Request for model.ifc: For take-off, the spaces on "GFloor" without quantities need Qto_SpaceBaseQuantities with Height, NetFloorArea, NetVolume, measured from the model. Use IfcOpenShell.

First a look at what the model holds.

```python
import ifcopenshell
import ifcopenshell.util.element
import ifcopenshell.util.unit

model = ifcopenshell.open("model.ifc")
print(model.schema)
for unit_type in ("LENGTHUNIT", "AREAUNIT", "VOLUMEUNIT"):
    print(unit_type, ifcopenshell.util.unit.calculate_unit_scale(model, unit_type))
storey = next(s for s in model.by_type("IfcBuildingStorey") if s.Name == "GFloor")
spaces = [e for e in ifcopenshell.util.element.get_decomposition(storey) if e.is_a("IfcSpace")]
for e in sorted(spaces, key=lambda e: e.id()):
    print(e.id(), e.is_a(), e.Name, list(ifcopenshell.util.element.get_psets(e, qtos_only=True)), sep=" | ")
```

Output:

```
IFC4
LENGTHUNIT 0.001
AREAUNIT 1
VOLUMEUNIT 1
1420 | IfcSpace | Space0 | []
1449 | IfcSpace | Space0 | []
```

```python
import ifcopenshell
import ifcopenshell.api.pset
import ifcopenshell.geom
import ifcopenshell.util.element
import ifcopenshell.util.shape
import ifcopenshell.util.unit

model = ifcopenshell.open("model.ifc")
unit_scale = ifcopenshell.util.unit.calculate_unit_scale(model)
area_scale = ifcopenshell.util.unit.calculate_unit_scale(model, "AREAUNIT")
volume_scale = ifcopenshell.util.unit.calculate_unit_scale(model, "VOLUMEUNIT")
settings = ifcopenshell.geom.settings()

storey = next(s for s in model.by_type("IfcBuildingStorey") if s.Name == "GFloor")
spaces = [e for e in ifcopenshell.util.element.get_decomposition(storey) if e.is_a("IfcSpace")]

for e in sorted(spaces, key=lambda e: e.id()):
    if ifcopenshell.util.element.get_psets(e, qtos_only=True, should_inherit=False):
        continue
    # Geometry comes back in metres, in the element's own axes.
    shape = ifcopenshell.geom.create_shape(settings, e)
    values = {
        "Height": ifcopenshell.util.shape.get_z(shape.geometry) / unit_scale,
        "NetFloorArea": ifcopenshell.util.shape.get_footprint_area(shape.geometry) / area_scale,
        "NetVolume": ifcopenshell.util.shape.get_volume(shape.geometry) / volume_scale,
    }
    qto = ifcopenshell.api.pset.add_qto(model, product=e, name="Qto_SpaceBaseQuantities")
    ifcopenshell.api.pset.edit_qto(model, qto=qto, properties=values)
    print(e.id(), {k: round(v, 3) for k, v in values.items()})

model.write("model-out.ifc")
```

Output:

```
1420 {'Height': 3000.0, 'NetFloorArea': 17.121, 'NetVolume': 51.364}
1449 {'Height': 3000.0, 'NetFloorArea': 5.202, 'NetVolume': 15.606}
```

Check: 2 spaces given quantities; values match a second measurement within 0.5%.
